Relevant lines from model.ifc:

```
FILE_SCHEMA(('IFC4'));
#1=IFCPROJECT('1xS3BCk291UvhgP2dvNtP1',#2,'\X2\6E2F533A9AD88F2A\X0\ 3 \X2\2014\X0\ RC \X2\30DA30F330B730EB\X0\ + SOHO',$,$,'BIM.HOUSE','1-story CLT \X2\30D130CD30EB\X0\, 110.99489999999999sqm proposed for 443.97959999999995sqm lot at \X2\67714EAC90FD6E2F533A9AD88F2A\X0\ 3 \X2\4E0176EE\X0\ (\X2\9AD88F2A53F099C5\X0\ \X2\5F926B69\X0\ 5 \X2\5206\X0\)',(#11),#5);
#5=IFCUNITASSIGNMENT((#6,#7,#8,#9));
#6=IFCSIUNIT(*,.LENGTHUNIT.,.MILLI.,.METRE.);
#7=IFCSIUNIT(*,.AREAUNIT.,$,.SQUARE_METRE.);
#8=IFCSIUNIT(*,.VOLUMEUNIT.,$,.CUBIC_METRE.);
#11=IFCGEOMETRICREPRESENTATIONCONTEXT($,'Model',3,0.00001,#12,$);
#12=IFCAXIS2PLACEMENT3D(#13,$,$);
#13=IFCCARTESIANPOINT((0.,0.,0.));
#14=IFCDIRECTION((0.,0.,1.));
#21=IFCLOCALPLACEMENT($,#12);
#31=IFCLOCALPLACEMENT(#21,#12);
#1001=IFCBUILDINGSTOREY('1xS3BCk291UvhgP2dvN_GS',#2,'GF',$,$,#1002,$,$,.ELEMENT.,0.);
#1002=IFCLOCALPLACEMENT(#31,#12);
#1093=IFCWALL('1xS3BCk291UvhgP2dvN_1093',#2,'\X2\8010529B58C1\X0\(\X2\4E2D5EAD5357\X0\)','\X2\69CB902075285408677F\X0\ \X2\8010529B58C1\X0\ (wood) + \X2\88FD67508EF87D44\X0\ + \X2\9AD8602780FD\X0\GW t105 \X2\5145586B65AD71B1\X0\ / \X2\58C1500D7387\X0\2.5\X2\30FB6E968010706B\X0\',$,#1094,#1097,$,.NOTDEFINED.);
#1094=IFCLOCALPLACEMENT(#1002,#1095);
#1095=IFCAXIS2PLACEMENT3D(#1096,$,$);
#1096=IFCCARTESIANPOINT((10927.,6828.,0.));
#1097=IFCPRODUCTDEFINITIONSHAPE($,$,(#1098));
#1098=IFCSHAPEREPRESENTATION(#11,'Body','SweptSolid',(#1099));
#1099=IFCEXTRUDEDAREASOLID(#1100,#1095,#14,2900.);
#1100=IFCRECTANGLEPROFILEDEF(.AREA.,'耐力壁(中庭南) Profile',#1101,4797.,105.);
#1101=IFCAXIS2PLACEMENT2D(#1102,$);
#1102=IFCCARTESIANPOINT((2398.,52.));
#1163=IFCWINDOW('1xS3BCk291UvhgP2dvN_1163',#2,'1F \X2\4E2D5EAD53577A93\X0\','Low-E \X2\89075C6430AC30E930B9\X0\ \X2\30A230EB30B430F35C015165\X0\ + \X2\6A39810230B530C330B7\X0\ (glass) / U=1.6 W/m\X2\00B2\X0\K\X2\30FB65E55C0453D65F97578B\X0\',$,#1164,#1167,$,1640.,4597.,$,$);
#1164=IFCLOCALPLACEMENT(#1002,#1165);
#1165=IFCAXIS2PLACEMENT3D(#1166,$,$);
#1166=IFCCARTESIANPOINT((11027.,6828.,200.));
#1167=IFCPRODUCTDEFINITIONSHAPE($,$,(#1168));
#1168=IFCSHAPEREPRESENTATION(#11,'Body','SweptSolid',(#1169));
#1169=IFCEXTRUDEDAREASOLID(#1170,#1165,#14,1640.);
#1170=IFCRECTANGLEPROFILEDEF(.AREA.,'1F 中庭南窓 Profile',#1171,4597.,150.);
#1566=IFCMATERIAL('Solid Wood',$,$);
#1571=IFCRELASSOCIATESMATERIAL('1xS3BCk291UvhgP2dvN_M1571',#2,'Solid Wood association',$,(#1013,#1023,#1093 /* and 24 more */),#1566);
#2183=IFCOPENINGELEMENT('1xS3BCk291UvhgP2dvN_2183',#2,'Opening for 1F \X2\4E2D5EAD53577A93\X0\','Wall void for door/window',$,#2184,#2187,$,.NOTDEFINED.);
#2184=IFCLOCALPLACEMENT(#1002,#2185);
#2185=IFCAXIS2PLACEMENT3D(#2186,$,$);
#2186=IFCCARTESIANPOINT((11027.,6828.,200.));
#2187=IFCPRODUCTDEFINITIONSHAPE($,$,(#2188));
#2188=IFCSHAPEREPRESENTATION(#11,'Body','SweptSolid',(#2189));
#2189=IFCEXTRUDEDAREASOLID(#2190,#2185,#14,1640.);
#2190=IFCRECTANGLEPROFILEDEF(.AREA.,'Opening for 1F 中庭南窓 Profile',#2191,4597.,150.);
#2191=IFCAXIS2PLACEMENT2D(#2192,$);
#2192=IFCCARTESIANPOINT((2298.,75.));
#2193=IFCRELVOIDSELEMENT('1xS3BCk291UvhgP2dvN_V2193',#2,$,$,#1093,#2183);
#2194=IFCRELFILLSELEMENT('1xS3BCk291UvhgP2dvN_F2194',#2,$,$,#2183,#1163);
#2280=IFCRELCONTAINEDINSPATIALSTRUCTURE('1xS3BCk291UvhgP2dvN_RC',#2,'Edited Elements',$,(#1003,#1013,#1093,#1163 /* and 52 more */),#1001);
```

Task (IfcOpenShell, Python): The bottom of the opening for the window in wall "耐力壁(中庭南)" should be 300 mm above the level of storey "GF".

```python
import numpy as np
import ifcopenshell
import ifcopenshell.api.geometry
import ifcopenshell.geom
import ifcopenshell.util.element
import ifcopenshell.util.placement
import ifcopenshell.util.shape
import ifcopenshell.util.unit

model = ifcopenshell.open("model.ifc")
unit_scale = ifcopenshell.util.unit.calculate_unit_scale(model)

window = model.by_guid("1xS3BCk291UvhgP2dvN_1163")
opening = window.FillsVoids[0].RelatingOpeningElement
storey = ifcopenshell.util.element.get_container(window, ifc_class="IfcBuildingStorey")
level = ifcopenshell.util.placement.get_local_placement(storey.ObjectPlacement)[2, 3]

# The opening's origin need not be at the sill, so measure its lowest point.
shape = ifcopenshell.geom.create_shape(ifcopenshell.geom.settings(), opening)
bottom = ifcopenshell.util.shape.get_shape_bottom_elevation(shape, shape.geometry) / unit_scale
dz = level + 300.0 - bottom

shift = np.array([0.0, 0.0, dz])
# The window is not placed relative to its opening, so move both.
for product in (opening, window):
    matrix = ifcopenshell.util.placement.get_local_placement(product.ObjectPlacement)
    matrix[:3, 3] += shift
    ifcopenshell.api.geometry.edit_object_placement(model, product=product, matrix=matrix, is_si=False)

print(f"moved by {dz * unit_scale:+.3f} m")

model.write("model_v2.ifc")
```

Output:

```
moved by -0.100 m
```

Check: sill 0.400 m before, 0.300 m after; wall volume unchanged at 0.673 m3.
